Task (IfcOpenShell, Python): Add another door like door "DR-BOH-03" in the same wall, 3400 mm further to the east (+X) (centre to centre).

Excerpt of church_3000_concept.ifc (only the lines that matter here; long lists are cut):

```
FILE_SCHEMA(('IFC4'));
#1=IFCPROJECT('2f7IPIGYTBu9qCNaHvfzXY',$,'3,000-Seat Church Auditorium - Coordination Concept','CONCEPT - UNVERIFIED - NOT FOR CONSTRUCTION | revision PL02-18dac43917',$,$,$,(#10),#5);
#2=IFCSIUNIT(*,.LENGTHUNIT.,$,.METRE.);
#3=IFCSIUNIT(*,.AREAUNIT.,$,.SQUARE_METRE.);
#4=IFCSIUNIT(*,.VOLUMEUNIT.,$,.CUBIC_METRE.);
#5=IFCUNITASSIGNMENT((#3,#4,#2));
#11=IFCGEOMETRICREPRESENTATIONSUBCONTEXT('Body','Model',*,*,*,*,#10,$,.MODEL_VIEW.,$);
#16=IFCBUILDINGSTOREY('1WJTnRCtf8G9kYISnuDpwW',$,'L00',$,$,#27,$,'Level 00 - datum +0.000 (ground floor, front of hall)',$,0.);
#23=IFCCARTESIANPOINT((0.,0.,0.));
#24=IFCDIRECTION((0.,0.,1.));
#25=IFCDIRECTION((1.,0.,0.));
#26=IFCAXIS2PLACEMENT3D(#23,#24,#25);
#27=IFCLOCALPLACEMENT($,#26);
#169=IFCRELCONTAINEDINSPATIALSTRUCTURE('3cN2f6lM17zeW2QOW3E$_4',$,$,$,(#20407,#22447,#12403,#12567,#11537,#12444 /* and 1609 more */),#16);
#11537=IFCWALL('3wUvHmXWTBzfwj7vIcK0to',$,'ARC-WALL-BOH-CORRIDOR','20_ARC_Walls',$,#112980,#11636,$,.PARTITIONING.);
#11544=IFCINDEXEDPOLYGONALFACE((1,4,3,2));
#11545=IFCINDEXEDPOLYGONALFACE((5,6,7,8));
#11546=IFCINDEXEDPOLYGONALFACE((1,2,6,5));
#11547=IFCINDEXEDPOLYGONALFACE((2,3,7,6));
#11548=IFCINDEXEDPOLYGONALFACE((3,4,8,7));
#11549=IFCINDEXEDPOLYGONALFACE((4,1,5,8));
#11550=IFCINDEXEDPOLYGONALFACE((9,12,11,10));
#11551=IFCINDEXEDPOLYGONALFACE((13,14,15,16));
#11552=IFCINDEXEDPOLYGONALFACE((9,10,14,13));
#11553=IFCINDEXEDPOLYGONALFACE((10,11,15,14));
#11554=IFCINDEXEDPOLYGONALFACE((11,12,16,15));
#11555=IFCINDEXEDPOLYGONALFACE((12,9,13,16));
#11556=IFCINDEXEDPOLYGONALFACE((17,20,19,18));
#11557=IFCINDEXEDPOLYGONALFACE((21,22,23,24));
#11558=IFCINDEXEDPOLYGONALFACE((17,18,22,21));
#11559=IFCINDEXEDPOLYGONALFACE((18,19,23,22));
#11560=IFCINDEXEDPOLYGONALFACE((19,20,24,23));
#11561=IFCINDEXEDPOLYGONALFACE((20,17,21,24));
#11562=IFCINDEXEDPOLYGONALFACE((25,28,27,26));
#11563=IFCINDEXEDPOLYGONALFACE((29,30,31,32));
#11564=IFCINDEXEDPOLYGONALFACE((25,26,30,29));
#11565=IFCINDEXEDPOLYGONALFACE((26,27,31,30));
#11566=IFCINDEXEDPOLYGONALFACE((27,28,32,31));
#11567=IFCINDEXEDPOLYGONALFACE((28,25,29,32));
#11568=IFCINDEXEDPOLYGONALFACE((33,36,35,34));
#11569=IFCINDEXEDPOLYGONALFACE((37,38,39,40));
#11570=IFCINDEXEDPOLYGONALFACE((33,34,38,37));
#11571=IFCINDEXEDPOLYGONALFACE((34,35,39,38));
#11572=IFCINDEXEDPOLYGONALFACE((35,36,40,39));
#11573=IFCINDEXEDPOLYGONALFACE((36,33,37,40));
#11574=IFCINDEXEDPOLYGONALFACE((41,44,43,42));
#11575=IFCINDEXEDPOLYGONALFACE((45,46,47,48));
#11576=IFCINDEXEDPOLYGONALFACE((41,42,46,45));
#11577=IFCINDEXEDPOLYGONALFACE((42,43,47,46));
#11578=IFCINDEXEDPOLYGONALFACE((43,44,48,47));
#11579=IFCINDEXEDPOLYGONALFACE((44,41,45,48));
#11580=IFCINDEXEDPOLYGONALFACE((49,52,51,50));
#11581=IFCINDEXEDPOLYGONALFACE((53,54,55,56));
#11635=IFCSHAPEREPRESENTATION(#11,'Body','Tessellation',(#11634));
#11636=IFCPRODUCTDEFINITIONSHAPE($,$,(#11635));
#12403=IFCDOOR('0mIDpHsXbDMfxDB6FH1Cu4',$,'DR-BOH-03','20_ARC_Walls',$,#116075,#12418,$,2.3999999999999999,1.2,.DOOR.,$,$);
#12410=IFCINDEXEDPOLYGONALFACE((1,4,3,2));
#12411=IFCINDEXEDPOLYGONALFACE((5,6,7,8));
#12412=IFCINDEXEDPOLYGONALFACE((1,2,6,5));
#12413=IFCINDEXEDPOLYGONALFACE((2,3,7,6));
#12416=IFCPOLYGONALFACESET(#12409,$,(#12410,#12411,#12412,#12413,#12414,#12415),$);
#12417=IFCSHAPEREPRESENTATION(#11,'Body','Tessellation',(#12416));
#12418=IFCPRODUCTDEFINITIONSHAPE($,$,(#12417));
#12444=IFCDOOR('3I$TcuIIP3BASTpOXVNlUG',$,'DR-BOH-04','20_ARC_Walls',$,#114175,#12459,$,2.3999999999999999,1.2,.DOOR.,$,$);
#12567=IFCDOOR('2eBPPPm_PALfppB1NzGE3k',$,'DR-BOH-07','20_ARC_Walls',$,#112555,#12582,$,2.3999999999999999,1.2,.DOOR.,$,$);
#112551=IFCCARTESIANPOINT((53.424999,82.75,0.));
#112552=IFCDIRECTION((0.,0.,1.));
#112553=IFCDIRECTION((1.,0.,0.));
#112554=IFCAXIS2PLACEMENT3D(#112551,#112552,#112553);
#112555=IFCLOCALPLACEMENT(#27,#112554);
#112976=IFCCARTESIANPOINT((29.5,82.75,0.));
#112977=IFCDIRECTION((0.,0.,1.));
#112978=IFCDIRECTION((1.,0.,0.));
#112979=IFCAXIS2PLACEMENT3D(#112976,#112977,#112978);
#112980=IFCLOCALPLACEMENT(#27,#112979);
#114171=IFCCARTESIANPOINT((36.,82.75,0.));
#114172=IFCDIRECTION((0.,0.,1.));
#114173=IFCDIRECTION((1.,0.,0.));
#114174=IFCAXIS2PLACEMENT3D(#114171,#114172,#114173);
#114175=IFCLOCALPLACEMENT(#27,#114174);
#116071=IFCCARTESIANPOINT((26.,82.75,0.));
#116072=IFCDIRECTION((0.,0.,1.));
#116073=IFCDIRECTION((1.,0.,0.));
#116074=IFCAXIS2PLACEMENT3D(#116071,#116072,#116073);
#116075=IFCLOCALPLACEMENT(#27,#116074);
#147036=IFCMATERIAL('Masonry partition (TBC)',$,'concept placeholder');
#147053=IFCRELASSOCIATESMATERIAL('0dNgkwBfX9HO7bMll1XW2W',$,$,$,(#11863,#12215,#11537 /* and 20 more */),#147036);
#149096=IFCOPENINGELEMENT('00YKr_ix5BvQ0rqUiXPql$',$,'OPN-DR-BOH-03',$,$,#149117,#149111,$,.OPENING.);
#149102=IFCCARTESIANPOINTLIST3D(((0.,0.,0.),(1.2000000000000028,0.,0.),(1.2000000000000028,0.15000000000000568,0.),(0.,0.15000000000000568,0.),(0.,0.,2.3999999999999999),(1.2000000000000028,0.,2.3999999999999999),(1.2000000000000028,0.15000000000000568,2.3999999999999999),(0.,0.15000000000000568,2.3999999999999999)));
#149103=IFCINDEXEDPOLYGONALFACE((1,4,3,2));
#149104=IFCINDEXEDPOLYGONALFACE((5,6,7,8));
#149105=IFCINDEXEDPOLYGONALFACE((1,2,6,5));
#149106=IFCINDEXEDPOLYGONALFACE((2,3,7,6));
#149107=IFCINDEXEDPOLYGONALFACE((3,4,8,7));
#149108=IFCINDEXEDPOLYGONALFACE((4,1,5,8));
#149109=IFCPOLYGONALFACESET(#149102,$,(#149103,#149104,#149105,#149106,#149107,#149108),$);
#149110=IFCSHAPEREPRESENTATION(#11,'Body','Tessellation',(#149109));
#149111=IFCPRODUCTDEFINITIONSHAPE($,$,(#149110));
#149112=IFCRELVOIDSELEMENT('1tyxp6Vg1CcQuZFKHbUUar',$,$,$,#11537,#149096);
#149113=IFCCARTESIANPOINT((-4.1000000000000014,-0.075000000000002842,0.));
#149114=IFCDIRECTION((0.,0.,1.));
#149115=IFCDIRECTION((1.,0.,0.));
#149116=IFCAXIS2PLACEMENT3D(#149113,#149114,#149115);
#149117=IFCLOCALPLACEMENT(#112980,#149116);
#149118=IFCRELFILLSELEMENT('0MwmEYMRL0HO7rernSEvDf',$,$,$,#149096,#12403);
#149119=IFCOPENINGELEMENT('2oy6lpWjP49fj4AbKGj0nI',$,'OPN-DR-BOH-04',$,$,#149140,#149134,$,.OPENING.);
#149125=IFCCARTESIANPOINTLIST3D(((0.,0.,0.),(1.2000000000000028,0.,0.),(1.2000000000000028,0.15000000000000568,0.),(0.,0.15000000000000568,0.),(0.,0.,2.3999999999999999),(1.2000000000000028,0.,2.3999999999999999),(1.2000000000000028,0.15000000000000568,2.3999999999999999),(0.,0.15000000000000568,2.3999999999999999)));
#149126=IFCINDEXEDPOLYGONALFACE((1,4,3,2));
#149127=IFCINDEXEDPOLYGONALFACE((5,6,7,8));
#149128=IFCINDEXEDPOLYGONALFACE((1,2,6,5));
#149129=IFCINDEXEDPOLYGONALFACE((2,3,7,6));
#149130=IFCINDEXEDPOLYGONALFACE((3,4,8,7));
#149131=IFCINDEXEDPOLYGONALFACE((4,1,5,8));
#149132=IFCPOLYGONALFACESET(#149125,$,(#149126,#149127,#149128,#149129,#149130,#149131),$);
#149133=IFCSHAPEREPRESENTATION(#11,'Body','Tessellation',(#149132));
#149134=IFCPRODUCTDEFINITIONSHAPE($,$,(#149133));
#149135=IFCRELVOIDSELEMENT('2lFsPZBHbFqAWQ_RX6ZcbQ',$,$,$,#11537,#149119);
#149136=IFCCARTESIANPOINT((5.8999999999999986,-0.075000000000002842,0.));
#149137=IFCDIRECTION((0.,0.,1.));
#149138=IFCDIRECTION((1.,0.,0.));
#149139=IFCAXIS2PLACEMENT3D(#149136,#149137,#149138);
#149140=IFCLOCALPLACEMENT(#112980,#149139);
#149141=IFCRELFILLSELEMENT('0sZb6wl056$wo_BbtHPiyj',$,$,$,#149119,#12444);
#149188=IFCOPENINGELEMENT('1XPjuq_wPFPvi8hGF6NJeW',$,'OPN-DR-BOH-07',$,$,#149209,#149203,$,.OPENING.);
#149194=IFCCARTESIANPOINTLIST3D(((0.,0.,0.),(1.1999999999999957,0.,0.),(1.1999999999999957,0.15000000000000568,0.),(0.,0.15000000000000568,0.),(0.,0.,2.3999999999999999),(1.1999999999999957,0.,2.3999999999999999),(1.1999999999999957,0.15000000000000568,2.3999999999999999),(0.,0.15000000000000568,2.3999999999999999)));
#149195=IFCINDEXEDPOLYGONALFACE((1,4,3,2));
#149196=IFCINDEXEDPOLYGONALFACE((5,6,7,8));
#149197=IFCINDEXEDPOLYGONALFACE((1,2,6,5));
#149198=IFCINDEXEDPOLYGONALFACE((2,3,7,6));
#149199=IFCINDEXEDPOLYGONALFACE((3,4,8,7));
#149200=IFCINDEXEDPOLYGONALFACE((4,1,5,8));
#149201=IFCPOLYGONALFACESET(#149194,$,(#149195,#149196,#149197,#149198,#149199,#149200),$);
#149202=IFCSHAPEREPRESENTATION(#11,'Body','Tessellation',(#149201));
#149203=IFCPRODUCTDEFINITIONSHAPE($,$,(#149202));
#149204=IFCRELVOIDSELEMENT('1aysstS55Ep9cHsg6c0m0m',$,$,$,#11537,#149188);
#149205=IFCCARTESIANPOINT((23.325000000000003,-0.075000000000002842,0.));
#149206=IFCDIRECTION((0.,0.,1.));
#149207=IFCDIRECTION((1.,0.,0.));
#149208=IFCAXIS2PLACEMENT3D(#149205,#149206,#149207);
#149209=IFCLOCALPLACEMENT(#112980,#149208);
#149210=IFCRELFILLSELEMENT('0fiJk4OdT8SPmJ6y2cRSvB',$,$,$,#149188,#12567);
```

```python
import ifcopenshell
import ifcopenshell.api.feature
import ifcopenshell.api.geometry
import ifcopenshell.api.root
import ifcopenshell.geom
import ifcopenshell.util.element
import ifcopenshell.util.placement
import ifcopenshell.util.shape

model = ifcopenshell.open("church_3000_concept.ifc")
settings = ifcopenshell.geom.settings()


def volume(element):
    """Net volume in cubic metres, openings subtracted."""
    shape = ifcopenshell.geom.create_shape(settings, element)
    return ifcopenshell.util.shape.get_volume(shape.geometry)


door = model.by_id(12403)
opening = door.FillsVoids[0].RelatingOpeningElement
wall = opening.VoidsElements[0].RelatingBuildingElement
before = volume(wall)
shift = ifcopenshell.util.placement.get_local_placement(wall.ObjectPlacement)[:3, 0] * 3.4

# copy_class copies the void relationship, type, container and properties, but no geometry.
new_opening = ifcopenshell.api.root.copy_class(model, product=opening)
new_opening.Representation = ifcopenshell.util.element.copy_deep(
    model, opening.Representation, exclude=["IfcGeometricRepresentationContext", "IfcRepresentationMap"]
)
new_door = ifcopenshell.api.root.copy_class(model, product=door)
new_door.Representation = ifcopenshell.util.element.copy_deep(
    model, door.Representation, exclude=["IfcGeometricRepresentationContext", "IfcRepresentationMap"]
)
ifcopenshell.api.feature.add_filling(model, opening=new_opening, element=new_door)

for old, new in ((opening, new_opening), (door, new_door)):
    matrix = ifcopenshell.util.placement.get_local_placement(old.ObjectPlacement)
    matrix[:3, 3] += shift
    ifcopenshell.api.geometry.edit_object_placement(model, product=new, matrix=matrix, is_si=False)

after = volume(wall)

print(f"wall volume {before:.3f} -> {after:.3f} m3")

model.write("church_3000_concept_rev.ifc")
```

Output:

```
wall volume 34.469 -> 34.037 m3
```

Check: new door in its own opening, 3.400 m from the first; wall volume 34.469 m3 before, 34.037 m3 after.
